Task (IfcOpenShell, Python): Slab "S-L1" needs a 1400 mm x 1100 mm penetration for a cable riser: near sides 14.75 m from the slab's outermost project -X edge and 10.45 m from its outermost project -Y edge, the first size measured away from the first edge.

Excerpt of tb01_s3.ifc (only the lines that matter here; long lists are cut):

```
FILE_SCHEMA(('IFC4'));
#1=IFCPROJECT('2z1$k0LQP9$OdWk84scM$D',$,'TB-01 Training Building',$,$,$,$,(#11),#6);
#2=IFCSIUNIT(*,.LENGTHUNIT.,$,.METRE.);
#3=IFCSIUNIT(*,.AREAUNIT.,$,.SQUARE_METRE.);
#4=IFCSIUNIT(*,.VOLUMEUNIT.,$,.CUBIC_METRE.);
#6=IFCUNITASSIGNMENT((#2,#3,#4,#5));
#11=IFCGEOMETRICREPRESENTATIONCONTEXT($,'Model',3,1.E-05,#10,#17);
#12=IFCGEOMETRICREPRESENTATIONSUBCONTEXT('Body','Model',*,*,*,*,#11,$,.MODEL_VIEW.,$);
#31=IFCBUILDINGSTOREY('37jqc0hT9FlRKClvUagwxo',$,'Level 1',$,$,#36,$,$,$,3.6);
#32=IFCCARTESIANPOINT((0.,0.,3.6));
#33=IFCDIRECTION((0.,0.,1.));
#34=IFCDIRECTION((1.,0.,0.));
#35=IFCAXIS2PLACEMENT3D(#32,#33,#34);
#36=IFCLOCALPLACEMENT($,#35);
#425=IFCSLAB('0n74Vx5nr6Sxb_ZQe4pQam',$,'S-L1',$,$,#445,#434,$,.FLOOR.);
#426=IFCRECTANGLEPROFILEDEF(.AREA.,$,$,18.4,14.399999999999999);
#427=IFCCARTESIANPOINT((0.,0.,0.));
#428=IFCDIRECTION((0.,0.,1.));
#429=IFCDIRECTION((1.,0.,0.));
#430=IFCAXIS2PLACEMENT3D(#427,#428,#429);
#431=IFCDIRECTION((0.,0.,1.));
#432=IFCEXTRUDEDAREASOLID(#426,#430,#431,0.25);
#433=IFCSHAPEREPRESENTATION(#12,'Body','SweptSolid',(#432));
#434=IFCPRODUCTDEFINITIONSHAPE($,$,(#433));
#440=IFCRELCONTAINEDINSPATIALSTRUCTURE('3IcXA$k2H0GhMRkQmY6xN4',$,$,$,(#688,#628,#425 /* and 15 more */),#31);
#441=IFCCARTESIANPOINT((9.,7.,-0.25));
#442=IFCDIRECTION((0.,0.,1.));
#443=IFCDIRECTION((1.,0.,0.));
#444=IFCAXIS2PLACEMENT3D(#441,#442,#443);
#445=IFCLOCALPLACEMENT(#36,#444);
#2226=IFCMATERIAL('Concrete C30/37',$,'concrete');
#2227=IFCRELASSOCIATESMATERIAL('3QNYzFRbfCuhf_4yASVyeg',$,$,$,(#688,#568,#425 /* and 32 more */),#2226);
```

```python
import numpy as np
import ifcopenshell
import ifcopenshell.api.feature
import ifcopenshell.api.geometry
import ifcopenshell.api.root
import ifcopenshell.geom
import ifcopenshell.util.placement
import ifcopenshell.util.representation
import ifcopenshell.util.shape
import ifcopenshell.util.unit

model = ifcopenshell.open("tb01_s3.ifc")
unit_scale = ifcopenshell.util.unit.calculate_unit_scale(model)
settings = ifcopenshell.geom.settings()


def volume(element):
    """Net volume in cubic metres, openings subtracted."""
    shape = ifcopenshell.geom.create_shape(settings, element)
    return ifcopenshell.util.shape.get_volume(shape.geometry)


slab = model.by_id(425)
before = volume(slab)

# Extent in the slab's own axes, in metres. The edges named are its -X and -Y sides.
slab_shape = ifcopenshell.geom.create_shape(settings, slab)
vertices = ifcopenshell.util.shape.get_vertices(slab_shape.geometry)
x_min, y_min, bottom = vertices.min(axis=0)
top = vertices[:, 2].max()

opening = ifcopenshell.api.root.create_entity(model, ifc_class="IfcOpeningElement", name="Cable riser opening", predefined_type="OPENING")
context = ifcopenshell.util.representation.get_context(model, "Model", "Body", "MODEL_VIEW")
width, depth = 1.4, 1.1
outline = [(0.0, 0.0), (width, 0.0), (width, depth), (0.0, depth), (0.0, 0.0)]
# Overshoot both faces by 50 mm so the cut is clean.
shape = ifcopenshell.api.geometry.add_slab_representation(
    model, context=context, depth=top - bottom + 0.1, polyline=outline
)
ifcopenshell.api.geometry.assign_representation(model, product=opening, representation=shape)

matrix = ifcopenshell.util.placement.get_local_placement(slab.ObjectPlacement)
matrix[:, 3] = matrix @ np.append(np.array([x_min + 14.75, y_min + 10.45, bottom - 0.05]) / unit_scale, 1.0)
ifcopenshell.api.geometry.edit_object_placement(model, product=opening, matrix=matrix, is_si=False)
ifcopenshell.api.feature.add_feature(model, feature=opening, element=slab)

after = volume(slab)

print(f"slab volume {before:.3f} -> {after:.3f} m3")

model.write("tb01_s3_edited.ifc")
```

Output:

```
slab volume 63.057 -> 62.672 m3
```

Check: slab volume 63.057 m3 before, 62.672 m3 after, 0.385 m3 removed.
